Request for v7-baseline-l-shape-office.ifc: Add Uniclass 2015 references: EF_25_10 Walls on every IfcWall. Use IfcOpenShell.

First a look at what the model holds.

```python
import ifcopenshell

model = ifcopenshell.open("v7-baseline-l-shape-office.ifc")
print(model.schema)
print("classifications:", [c.Name for c in model.by_type("IfcClassification")])
for ifc_class in ("IfcDoor", "IfcRoof", "IfcStair", "IfcWall", "IfcWindow"):
    print(ifc_class, len(model.by_type(ifc_class)))
```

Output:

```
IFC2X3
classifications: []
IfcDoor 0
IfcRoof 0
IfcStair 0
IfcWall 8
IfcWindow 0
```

```python
import ifcopenshell
import ifcopenshell.api.classification

model = ifcopenshell.open("v7-baseline-l-shape-office.ifc")

# IFC2X3 requires Source and Edition and has no link from the project to the system.
system = model.create_entity("IfcClassification", Source="NBS", Edition="2015", Name="Uniclass 2015")

codes = {
    "IfcWall": ("EF_25_10", "Walls"),
}
for ifc_class, (code, name) in codes.items():
    products = model.by_type(ifc_class)
    ifcopenshell.api.classification.add_reference(
        model, products=products, classification=system, identification=code, name=name
    )
    print(code, len(products))

model.write("v7-baseline-l-shape-office_edited.ifc")
```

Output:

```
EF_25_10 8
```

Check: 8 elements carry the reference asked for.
